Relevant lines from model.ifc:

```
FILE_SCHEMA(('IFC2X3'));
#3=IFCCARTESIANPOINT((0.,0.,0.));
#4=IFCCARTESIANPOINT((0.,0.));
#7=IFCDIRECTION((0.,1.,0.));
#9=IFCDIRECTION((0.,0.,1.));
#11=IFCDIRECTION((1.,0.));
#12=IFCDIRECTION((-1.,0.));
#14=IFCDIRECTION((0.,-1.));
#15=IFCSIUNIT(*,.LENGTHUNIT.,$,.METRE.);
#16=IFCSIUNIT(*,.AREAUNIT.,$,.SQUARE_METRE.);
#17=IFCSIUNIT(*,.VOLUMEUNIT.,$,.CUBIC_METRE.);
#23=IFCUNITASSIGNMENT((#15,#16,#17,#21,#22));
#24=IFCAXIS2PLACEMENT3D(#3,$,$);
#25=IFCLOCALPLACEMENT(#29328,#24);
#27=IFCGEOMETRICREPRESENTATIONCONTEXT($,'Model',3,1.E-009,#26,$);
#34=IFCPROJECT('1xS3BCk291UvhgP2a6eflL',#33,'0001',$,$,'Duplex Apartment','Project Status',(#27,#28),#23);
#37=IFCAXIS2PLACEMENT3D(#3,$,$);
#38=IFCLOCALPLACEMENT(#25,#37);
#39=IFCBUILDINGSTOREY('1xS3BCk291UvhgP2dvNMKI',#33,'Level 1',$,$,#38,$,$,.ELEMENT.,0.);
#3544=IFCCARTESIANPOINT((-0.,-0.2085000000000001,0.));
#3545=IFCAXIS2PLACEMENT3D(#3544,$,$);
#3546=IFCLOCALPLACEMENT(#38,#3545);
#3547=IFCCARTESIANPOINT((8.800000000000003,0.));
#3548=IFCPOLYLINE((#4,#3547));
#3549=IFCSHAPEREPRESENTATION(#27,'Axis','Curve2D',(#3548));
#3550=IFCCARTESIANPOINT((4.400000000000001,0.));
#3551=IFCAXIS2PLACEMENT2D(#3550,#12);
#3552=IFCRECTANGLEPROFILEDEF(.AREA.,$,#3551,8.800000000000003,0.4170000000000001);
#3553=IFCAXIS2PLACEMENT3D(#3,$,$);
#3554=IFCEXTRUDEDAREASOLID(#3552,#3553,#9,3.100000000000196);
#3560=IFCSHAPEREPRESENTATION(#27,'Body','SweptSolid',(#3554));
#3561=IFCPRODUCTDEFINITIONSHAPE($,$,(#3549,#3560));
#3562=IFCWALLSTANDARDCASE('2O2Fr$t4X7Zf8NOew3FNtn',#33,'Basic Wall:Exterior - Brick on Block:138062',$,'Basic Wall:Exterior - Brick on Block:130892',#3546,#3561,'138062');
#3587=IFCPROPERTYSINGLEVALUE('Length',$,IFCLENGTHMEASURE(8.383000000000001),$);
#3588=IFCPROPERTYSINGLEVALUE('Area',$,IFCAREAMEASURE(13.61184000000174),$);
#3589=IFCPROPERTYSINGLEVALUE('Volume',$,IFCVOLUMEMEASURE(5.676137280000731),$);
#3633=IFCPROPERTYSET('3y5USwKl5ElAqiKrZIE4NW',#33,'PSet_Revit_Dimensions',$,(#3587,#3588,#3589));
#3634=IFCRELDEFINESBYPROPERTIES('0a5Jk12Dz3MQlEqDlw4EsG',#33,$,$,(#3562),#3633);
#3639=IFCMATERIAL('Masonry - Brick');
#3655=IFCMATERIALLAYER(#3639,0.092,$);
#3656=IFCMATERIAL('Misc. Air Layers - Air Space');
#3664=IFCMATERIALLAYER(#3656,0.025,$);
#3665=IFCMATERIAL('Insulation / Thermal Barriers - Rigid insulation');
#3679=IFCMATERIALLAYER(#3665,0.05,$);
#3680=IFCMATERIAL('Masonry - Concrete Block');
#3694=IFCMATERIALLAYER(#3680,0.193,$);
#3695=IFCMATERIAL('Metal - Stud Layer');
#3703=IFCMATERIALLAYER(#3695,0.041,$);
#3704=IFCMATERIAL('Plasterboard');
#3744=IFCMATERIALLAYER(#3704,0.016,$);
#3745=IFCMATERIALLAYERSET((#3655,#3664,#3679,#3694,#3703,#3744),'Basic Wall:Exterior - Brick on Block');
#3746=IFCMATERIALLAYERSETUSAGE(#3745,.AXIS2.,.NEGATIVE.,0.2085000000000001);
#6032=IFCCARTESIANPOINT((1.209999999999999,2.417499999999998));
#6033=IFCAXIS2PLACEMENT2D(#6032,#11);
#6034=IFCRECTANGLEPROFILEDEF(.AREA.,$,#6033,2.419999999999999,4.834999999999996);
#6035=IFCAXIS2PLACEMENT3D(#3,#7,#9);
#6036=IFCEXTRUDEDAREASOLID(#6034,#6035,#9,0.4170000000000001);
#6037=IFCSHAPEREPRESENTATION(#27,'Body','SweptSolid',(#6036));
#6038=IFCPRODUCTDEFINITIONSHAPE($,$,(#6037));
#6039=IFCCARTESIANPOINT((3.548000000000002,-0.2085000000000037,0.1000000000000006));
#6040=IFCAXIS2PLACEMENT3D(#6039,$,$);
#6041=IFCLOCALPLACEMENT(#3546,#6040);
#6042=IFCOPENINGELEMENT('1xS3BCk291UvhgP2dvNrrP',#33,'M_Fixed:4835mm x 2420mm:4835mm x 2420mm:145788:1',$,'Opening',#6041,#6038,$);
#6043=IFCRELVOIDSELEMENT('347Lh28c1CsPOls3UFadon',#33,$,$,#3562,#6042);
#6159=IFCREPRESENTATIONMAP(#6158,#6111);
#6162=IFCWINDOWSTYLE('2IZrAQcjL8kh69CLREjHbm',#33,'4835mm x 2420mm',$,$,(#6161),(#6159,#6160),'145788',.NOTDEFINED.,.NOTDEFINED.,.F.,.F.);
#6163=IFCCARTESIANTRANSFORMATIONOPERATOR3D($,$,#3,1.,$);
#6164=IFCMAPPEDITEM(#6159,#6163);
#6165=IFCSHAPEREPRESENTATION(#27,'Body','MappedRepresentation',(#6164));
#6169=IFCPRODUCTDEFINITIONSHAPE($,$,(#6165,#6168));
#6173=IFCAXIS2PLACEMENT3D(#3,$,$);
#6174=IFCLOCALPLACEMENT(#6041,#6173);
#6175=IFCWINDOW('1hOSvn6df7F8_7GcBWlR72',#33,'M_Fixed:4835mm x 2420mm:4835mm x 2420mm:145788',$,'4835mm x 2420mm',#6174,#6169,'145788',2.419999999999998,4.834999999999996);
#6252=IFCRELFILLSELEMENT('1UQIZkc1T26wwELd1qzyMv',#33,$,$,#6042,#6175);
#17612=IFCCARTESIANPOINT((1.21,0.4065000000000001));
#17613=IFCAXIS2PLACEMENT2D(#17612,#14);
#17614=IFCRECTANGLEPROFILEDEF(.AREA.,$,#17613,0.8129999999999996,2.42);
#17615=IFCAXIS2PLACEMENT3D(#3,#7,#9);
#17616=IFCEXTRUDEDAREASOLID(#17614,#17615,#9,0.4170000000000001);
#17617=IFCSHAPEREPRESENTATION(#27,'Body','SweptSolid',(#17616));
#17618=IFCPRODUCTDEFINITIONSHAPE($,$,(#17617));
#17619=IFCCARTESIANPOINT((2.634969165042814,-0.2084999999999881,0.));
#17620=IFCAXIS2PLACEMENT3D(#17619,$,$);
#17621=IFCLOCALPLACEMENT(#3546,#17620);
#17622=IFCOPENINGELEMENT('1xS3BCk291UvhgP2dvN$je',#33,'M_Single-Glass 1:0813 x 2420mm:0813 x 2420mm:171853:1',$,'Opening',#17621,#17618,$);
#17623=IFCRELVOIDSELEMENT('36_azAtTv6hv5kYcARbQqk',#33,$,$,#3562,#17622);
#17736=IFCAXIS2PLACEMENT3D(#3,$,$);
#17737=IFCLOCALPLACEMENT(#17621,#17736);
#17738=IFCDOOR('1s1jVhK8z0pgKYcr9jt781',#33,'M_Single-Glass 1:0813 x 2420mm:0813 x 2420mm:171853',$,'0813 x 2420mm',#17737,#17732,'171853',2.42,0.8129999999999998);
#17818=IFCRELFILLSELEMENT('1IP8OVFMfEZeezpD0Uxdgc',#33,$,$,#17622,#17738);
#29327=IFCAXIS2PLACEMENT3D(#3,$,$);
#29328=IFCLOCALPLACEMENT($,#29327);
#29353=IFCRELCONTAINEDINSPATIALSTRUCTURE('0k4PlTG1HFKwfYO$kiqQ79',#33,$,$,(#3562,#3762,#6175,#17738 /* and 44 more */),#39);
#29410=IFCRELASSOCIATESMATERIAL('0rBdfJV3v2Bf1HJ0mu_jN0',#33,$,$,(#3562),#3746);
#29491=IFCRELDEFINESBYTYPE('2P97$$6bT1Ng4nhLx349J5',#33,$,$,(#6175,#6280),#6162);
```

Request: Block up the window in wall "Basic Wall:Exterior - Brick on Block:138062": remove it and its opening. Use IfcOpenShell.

```python
import ifcopenshell
import ifcopenshell.api.feature
import ifcopenshell.api.pset
import ifcopenshell.api.root
import ifcopenshell.geom
import ifcopenshell.util.element
import ifcopenshell.util.shape
import ifcopenshell.util.unit

model = ifcopenshell.open("model.ifc")
area_scale = ifcopenshell.util.unit.calculate_unit_scale(model, "AREAUNIT")
volume_scale = ifcopenshell.util.unit.calculate_unit_scale(model, "VOLUMEUNIT")
settings = ifcopenshell.geom.settings()


def volume(element):
    """Net volume in cubic metres, openings subtracted."""
    shape = ifcopenshell.geom.create_shape(settings, element)
    return ifcopenshell.util.shape.get_volume(shape.geometry)


window = model.by_guid("1hOSvn6df7F8_7GcBWlR72")
opening = window.FillsVoids[0].RelatingOpeningElement
wall = opening.VoidsElements[0].RelatingBuildingElement
before = volume(wall)

ifcopenshell.api.root.remove_product(model, product=window)
ifcopenshell.api.feature.remove_feature(model, feature=opening)

after = volume(wall)
thickness = 0.417  # wall thickness in metres

# Update the wall's stored quantities.
pset = model.by_id(ifcopenshell.util.element.get_pset(wall, "PSet_Revit_Dimensions", should_inherit=False)["id"])
ifcopenshell.api.pset.edit_pset(model, pset=pset, properties={
    "Area": model.create_entity("IfcAreaMeasure", after / thickness / area_scale),
    "Volume": model.create_entity("IfcVolumeMeasure", after / volume_scale),
})

print(f"wall volume {before:.3f} -> {after:.3f} m3")

model.write("model_v2.ifc")
```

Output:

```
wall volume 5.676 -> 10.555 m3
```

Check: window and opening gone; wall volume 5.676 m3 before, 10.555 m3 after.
